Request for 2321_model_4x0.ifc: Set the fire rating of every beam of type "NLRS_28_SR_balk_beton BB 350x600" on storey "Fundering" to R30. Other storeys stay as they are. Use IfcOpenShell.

First a look at what the model holds.

```python
import ifcopenshell
import ifcopenshell.util.element

model = ifcopenshell.open("2321_model_4x0.ifc")
print(model.schema)
storey = next(s for s in model.by_type("IfcBuildingStorey") if s.Name == "Fundering")
beams = [e for e in ifcopenshell.util.element.get_decomposition(storey) if e.is_a("IfcBeam")]
seen = {}
for e in beams:
    element_type = ifcopenshell.util.element.get_type(e)
    key = (element_type.Name if element_type != e and element_type else None, ifcopenshell.util.element.get_pset(e, "Pset_BeamCommon", "FireRating"))
    seen[key] = seen.get(key, 0) + 1
for (name, value), count in sorted(seen.items(), key=str):
    print(count, "x", name, "|", value)
```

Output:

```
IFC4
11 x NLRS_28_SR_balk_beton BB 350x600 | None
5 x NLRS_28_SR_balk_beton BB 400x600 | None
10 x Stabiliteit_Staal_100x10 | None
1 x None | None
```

```python
import ifcopenshell
import ifcopenshell.api.pset
import ifcopenshell.util.element

model = ifcopenshell.open("2321_model_4x0.ifc")

storey = next(s for s in model.by_type("IfcBuildingStorey") if s.Name == "Fundering")
beams = [e for e in ifcopenshell.util.element.get_decomposition(storey) if e.is_a("IfcBeam")]

count = 0
for e in beams:
    element_type = ifcopenshell.util.element.get_type(e)
    if element_type in (None, e) or element_type.Name != "NLRS_28_SR_balk_beton BB 350x600":
        continue
    # add_pset returns the element's existing set when there is one.
    pset = ifcopenshell.api.pset.add_pset(model, product=e, name="Pset_BeamCommon")
    ifcopenshell.api.pset.edit_pset(model, pset=pset, properties={"FireRating": "R30"})
    count += 1

print(count, "beams updated")

model.write("2321_model_4x0_rev.ifc")
```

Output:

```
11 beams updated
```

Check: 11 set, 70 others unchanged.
